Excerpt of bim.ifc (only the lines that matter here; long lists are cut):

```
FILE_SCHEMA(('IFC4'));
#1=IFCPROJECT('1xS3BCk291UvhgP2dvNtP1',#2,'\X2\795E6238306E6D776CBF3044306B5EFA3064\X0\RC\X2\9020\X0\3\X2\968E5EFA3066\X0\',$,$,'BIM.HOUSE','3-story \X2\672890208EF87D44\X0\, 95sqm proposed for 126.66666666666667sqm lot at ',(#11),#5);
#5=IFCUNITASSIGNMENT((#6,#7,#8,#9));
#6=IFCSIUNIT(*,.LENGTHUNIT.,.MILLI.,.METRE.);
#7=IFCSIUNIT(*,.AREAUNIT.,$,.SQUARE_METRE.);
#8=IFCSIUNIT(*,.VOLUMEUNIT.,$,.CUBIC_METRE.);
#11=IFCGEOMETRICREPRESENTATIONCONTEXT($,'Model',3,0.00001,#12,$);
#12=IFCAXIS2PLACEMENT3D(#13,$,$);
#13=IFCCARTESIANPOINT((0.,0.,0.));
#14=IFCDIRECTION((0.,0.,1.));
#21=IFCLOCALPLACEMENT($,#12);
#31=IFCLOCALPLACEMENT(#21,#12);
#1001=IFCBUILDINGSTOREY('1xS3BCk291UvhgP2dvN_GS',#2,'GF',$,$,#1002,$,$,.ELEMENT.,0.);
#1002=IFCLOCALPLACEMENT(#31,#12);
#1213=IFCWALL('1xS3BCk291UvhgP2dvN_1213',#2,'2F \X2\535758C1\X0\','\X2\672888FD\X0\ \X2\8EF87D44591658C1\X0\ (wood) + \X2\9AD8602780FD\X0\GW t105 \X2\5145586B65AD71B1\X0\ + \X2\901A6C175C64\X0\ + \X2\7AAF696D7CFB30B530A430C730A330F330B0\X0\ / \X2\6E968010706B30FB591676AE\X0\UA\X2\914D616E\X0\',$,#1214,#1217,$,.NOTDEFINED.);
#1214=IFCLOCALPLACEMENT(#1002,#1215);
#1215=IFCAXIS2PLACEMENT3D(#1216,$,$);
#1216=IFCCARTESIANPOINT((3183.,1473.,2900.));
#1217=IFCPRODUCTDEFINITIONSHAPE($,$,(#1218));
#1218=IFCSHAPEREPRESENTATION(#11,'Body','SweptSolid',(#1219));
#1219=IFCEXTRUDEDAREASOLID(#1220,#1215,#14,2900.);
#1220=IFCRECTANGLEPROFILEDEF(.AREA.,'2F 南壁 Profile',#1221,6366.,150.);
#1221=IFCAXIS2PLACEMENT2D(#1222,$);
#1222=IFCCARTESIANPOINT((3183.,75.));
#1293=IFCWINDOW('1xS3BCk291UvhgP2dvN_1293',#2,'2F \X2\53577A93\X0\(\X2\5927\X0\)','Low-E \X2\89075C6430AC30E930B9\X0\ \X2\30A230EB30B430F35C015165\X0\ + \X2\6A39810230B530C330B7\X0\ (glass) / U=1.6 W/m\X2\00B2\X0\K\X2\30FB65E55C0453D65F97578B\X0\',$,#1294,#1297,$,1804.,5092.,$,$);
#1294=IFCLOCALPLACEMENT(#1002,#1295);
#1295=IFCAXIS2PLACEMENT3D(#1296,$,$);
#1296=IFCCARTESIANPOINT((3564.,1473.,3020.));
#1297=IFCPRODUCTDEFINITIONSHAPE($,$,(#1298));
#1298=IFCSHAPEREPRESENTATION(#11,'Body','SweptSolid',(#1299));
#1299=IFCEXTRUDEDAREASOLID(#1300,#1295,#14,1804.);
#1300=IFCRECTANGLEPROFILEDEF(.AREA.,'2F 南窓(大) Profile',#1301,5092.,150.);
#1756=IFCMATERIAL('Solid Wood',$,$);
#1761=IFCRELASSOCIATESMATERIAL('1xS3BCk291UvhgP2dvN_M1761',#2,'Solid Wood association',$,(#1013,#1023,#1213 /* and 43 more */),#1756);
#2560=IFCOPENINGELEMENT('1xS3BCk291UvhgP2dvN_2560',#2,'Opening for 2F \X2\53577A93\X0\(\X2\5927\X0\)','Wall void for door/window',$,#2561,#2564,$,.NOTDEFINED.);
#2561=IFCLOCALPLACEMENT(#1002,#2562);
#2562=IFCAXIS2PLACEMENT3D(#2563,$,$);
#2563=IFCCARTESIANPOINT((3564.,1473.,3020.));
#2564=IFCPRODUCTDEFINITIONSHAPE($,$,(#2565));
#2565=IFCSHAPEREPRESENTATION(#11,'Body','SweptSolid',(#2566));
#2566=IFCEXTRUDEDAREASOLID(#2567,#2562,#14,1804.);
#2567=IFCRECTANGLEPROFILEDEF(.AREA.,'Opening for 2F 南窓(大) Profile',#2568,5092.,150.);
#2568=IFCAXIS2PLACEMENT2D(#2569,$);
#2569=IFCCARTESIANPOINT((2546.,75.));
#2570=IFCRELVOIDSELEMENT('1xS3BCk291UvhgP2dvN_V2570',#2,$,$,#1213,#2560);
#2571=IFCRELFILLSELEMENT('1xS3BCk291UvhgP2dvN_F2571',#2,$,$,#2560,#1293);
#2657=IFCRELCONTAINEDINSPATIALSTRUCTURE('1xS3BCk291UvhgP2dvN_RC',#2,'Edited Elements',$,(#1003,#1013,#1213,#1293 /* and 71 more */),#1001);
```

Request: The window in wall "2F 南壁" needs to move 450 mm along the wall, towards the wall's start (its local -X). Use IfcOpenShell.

```python
import ifcopenshell
import ifcopenshell.api.geometry
import ifcopenshell.util.placement

model = ifcopenshell.open("bim.ifc")

window = model.by_guid("1xS3BCk291UvhgP2dvN_1293")
opening = window.FillsVoids[0].RelatingOpeningElement
wall = opening.VoidsElements[0].RelatingBuildingElement

wall_matrix = ifcopenshell.util.placement.get_local_placement(wall.ObjectPlacement)
shift = wall_matrix[:3, 0] * -450.0
before = ifcopenshell.util.placement.get_local_placement(window.ObjectPlacement)[:3, 3].copy()

# The window is not placed relative to its opening, so move both.
for product in (opening, window):
    matrix = ifcopenshell.util.placement.get_local_placement(product.ObjectPlacement)
    matrix[:3, 3] += shift
    ifcopenshell.api.geometry.edit_object_placement(model, product=product, matrix=matrix, is_si=False)

after = ifcopenshell.util.placement.get_local_placement(window.ObjectPlacement)[:3, 3]
print("window moved by", (after - before).round(3) + 0.0)

model.write("bim_rev.ifc")
```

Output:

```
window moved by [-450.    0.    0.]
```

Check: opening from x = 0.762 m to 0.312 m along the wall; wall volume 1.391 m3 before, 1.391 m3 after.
